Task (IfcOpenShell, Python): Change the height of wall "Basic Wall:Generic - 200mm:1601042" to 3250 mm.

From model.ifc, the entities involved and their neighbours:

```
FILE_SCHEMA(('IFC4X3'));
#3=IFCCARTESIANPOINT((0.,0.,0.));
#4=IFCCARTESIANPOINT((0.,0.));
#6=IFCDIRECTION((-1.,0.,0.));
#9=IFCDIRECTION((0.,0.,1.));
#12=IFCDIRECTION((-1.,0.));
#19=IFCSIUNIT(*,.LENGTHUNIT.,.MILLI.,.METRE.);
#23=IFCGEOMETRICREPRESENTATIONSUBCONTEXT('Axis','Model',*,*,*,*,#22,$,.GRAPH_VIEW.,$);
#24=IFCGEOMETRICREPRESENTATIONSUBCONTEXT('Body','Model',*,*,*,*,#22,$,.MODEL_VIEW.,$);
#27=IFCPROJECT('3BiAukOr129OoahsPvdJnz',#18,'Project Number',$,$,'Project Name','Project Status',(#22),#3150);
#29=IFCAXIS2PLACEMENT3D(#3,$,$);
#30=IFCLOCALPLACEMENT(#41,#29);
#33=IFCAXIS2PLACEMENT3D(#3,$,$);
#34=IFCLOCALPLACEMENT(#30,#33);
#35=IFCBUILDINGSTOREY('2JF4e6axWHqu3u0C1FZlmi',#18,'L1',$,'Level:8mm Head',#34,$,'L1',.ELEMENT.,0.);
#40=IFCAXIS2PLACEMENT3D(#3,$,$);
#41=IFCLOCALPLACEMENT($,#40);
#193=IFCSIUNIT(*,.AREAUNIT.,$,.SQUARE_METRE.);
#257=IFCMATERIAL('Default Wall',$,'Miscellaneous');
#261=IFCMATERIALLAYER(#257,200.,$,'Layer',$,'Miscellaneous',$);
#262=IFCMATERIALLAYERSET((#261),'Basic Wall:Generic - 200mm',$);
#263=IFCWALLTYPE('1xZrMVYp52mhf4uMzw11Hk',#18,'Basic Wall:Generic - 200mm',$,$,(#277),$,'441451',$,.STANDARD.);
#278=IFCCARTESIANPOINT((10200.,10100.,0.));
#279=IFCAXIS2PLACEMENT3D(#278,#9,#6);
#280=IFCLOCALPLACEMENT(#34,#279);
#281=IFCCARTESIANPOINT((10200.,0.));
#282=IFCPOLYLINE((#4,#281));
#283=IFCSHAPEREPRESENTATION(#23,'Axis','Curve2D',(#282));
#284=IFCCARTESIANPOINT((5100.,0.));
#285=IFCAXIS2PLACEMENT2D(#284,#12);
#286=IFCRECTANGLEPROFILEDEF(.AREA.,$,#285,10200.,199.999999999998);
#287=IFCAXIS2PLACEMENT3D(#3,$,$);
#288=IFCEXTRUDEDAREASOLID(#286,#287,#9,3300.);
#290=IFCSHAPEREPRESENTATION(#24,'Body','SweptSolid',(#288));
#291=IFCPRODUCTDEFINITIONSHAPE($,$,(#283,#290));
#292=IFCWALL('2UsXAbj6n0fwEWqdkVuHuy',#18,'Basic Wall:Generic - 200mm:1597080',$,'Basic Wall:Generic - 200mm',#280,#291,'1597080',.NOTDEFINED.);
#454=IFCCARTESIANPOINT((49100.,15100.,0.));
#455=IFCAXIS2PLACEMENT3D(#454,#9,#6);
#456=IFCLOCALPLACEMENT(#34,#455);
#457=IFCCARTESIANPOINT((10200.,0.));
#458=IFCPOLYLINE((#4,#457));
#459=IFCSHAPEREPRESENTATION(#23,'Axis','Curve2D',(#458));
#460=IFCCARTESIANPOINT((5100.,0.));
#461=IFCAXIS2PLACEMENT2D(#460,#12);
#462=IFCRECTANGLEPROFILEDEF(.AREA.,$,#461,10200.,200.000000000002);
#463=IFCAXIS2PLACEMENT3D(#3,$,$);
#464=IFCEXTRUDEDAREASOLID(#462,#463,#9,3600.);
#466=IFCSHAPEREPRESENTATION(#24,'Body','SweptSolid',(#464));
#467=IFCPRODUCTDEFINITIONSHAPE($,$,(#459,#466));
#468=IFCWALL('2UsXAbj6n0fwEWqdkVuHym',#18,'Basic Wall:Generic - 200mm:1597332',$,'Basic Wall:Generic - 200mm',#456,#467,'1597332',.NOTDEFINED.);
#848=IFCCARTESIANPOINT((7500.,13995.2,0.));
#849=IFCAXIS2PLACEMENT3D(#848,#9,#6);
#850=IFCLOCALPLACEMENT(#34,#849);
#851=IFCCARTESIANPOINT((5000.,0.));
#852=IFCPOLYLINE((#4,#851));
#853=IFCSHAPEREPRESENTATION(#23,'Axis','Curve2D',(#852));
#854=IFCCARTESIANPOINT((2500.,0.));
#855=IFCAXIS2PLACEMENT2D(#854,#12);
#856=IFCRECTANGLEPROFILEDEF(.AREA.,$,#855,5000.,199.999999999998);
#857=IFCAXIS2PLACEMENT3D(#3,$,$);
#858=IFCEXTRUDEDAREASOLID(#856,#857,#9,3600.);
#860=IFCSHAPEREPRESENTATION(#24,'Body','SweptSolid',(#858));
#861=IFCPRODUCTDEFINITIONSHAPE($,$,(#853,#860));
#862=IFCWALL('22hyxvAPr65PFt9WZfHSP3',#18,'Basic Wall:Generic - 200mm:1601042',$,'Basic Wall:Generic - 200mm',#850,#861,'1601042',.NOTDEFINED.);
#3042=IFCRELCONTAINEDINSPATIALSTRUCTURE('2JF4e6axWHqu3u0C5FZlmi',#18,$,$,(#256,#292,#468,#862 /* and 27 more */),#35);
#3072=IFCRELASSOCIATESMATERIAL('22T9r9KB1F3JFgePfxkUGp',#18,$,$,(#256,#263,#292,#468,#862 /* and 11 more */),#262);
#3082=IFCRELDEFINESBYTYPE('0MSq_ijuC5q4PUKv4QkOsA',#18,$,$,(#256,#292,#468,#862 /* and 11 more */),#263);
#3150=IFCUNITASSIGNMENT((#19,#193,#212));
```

```python
import ifcopenshell
import ifcopenshell.geom
import ifcopenshell.util.representation
import ifcopenshell.util.shape
import ifcopenshell.util.unit

model = ifcopenshell.open("model.ifc")
unit_scale = ifcopenshell.util.unit.calculate_unit_scale(model)
settings = ifcopenshell.geom.settings()


def volume(element):
    """Net volume in cubic metres, openings subtracted."""
    shape = ifcopenshell.geom.create_shape(settings, element)
    return ifcopenshell.util.shape.get_volume(shape.geometry)


wall = model.by_guid("22hyxvAPr65PFt9WZfHSP3")
before = volume(wall)

body = ifcopenshell.util.representation.get_representation(wall, "Model", "Body")
solid = body.Items[0]
old_height = solid.Depth
solid.Depth = 3.25 / unit_scale
after = volume(wall)

print(f"height {old_height:g} -> {solid.Depth:g}, volume {before:.3f} -> {after:.3f} m3")

model.write("model-out.ifc")
```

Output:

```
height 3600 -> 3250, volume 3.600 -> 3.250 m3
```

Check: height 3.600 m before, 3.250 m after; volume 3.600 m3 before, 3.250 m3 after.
